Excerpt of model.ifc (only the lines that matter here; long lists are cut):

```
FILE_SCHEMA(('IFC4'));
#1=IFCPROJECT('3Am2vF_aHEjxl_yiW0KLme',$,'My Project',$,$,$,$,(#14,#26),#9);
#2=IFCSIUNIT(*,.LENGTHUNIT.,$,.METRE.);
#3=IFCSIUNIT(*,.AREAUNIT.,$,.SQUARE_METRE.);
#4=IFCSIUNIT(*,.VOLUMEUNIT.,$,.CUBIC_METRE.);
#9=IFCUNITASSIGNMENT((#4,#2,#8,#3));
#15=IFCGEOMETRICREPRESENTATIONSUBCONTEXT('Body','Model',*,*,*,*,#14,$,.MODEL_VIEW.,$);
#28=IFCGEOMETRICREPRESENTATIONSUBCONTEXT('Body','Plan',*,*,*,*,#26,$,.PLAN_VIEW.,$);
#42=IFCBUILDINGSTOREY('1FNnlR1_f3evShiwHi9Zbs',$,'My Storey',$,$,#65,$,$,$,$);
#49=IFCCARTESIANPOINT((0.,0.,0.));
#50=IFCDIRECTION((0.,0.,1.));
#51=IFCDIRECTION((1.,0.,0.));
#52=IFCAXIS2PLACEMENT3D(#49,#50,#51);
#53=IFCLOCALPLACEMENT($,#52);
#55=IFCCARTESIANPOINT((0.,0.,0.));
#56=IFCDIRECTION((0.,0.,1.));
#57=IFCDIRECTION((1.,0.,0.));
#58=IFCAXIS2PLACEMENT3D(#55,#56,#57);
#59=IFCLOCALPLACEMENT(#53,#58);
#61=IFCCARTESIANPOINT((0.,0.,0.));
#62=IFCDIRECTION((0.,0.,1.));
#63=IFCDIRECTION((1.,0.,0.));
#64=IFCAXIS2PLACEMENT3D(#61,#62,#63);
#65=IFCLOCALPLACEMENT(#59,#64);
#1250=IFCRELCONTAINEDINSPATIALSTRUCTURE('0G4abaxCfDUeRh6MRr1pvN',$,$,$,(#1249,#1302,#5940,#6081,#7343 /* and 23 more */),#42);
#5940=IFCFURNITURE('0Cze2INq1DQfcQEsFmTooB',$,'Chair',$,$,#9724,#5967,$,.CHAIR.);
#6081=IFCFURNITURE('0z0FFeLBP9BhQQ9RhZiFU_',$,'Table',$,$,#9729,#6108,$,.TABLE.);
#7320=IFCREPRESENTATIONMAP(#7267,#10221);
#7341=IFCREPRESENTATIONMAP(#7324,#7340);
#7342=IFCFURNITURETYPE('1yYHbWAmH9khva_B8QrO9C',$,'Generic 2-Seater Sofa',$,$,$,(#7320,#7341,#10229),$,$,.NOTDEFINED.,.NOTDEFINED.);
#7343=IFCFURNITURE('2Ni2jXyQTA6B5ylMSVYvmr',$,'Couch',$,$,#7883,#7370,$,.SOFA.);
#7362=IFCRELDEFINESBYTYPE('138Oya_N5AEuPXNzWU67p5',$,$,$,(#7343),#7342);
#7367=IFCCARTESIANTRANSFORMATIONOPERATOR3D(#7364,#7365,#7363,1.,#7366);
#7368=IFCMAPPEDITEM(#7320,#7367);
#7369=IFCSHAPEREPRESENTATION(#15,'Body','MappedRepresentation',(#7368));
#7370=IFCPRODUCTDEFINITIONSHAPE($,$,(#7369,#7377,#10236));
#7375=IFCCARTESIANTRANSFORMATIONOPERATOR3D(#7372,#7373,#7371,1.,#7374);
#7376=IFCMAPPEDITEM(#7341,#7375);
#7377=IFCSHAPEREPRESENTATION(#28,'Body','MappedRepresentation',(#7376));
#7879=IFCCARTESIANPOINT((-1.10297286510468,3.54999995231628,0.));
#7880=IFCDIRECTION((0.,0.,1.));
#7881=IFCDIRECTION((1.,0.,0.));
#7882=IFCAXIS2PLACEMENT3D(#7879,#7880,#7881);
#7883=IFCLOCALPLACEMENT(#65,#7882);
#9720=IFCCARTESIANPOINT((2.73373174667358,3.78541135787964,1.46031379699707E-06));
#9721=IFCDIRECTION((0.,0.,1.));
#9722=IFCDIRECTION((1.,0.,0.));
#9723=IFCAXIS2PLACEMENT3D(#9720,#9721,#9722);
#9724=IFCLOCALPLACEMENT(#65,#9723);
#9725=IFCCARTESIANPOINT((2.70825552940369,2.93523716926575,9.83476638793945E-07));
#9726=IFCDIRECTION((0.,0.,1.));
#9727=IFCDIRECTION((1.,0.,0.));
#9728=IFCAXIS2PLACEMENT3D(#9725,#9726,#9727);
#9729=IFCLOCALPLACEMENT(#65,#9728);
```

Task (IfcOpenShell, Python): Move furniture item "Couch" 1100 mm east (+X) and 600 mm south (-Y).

```python
import ifcopenshell
import ifcopenshell.api.geometry
import ifcopenshell.util.placement

model = ifcopenshell.open("model.ifc")

item = model.by_id(7343)
matrix = ifcopenshell.util.placement.get_local_placement(item.ObjectPlacement)
matrix[0, 3] += 1.1
matrix[1, 3] -= 0.6
ifcopenshell.api.geometry.edit_object_placement(model, product=item, matrix=matrix, is_si=False)

print(ifcopenshell.util.placement.get_local_placement(item.ObjectPlacement).round(3) + 0.0)

model.write("model_updated.ifc")
```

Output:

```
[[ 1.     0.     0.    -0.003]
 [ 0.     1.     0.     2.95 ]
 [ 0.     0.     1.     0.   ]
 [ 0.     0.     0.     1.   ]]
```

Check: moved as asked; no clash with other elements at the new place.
